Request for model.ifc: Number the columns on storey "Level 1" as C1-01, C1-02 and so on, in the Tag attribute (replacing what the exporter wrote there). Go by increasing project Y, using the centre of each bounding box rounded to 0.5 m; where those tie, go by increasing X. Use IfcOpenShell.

First a look at what the model holds.

```python
import ifcopenshell
import ifcopenshell.util.element
import ifcopenshell.util.placement

model = ifcopenshell.open("model.ifc")
print(model.schema)
storey = next(s for s in model.by_type("IfcBuildingStorey") if s.Name == "Level 1")
columns = [e for e in ifcopenshell.util.element.get_decomposition(storey) if e.is_a("IfcColumn")]
for e in sorted(columns, key=lambda e: e.id()):
    origin = ifcopenshell.util.placement.get_local_placement(e.ObjectPlacement)[:3, 3]
    print(e.id(), e.Tag, e.Name, origin.round(2) + 0.0, sep=" | ")
```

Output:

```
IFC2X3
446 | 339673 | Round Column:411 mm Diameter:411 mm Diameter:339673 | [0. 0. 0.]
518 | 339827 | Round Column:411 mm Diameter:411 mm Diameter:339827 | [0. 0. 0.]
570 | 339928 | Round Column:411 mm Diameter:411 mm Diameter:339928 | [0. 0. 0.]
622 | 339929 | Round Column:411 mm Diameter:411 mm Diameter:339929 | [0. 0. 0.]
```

```python
import ifcopenshell
import ifcopenshell.geom
import ifcopenshell.util.element
import ifcopenshell.util.shape

model = ifcopenshell.open("model.ifc")
settings = ifcopenshell.geom.settings()
settings.set("use-world-coords", True)


def centre(element):
    shape = ifcopenshell.geom.create_shape(settings, element)
    return ifcopenshell.util.shape.get_bbox_centroid(shape.geometry)


storey = next(s for s in model.by_type("IfcBuildingStorey") if s.Name == "Level 1")
columns = [e for e in ifcopenshell.util.element.get_decomposition(storey) if e.is_a("IfcColumn")]

# Insertion points can sit at a corner or the storey origin, so sort by the geometry (in metres).
centres = {e: centre(e) for e in columns}
columns.sort(key=lambda e: (round(centres[e][1] / 0.5), centres[e][0]))

for i, e in enumerate(columns, start=1):
    number = f"C1-{i:02d}"
    e.Tag = number
    print(e.id(), number)

model.write("model-out.ifc")
```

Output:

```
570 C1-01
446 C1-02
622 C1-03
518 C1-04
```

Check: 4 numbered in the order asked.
